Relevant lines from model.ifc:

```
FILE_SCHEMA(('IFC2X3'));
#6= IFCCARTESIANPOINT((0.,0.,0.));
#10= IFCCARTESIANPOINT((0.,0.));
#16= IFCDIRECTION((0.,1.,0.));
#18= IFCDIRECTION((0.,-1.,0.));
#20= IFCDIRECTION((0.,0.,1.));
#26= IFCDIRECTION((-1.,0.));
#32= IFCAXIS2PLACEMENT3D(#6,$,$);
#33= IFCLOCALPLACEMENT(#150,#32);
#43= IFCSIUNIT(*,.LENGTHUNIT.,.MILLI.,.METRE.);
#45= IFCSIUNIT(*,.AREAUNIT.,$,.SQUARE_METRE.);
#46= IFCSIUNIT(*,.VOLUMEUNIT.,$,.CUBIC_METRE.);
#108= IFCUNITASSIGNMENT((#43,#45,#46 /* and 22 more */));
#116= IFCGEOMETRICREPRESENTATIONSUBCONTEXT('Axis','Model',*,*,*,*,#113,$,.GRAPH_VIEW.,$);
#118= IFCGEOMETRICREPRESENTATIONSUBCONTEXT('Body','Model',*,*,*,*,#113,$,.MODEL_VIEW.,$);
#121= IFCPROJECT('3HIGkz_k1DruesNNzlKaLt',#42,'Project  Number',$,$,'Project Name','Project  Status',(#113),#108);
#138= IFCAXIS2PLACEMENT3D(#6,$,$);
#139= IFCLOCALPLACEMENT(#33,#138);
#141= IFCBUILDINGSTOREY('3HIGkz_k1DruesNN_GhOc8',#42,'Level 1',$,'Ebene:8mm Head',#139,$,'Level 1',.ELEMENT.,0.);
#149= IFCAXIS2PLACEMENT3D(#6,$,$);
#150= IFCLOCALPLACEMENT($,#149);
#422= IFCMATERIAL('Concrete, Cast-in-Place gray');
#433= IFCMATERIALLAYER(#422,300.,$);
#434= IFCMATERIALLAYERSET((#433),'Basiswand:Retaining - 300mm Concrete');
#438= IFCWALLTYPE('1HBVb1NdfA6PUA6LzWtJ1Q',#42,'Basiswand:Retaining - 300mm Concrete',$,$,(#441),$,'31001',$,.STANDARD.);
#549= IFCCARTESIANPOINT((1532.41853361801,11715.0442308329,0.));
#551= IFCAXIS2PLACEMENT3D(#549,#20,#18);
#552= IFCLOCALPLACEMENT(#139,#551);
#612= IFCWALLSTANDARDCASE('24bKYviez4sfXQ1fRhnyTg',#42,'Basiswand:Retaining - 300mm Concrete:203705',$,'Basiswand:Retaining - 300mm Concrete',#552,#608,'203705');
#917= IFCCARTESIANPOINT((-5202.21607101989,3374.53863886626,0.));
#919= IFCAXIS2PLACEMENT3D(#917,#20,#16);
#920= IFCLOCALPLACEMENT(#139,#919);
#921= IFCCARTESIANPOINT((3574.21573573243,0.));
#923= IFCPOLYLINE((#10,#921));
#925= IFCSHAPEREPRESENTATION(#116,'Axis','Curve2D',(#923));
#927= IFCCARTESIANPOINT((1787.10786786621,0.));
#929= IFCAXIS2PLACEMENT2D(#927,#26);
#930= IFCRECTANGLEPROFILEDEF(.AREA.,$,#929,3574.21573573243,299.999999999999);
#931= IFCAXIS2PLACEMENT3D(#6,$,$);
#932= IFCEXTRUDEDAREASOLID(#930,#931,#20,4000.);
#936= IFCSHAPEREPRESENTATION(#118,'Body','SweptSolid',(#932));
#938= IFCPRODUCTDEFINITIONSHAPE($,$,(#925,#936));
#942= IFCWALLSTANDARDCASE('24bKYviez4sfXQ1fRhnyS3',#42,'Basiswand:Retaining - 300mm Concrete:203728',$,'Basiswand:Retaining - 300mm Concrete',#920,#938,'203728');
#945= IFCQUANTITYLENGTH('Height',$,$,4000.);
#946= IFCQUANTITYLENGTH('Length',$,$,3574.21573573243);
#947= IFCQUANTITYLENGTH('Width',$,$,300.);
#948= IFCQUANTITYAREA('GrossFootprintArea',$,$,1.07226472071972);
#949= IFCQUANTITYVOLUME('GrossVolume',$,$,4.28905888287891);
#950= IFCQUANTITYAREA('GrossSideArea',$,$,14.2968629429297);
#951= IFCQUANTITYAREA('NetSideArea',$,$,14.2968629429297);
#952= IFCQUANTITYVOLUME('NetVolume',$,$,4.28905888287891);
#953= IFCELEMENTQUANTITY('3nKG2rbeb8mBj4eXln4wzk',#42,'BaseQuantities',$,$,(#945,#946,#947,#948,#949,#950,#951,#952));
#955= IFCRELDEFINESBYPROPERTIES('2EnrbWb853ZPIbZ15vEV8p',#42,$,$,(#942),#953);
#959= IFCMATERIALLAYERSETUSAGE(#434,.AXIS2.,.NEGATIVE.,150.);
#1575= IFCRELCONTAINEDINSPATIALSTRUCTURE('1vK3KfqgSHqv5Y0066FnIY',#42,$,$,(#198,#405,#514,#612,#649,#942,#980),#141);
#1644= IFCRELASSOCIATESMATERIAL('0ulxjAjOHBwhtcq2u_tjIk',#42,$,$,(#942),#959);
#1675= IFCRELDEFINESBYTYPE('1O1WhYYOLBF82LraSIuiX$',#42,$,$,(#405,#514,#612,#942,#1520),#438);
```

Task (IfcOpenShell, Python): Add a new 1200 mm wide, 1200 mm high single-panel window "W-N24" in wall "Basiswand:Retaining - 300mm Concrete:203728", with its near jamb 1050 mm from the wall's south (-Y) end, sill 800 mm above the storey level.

```python
import numpy as np
import ifcopenshell
import ifcopenshell.api.feature
import ifcopenshell.api.geometry
import ifcopenshell.api.pset
import ifcopenshell.api.root
import ifcopenshell.api.spatial
import ifcopenshell.api.type
import ifcopenshell.geom
import ifcopenshell.util.element
import ifcopenshell.util.placement
import ifcopenshell.util.representation
import ifcopenshell.util.shape
import ifcopenshell.util.unit

model = ifcopenshell.open("model.ifc")
unit_scale = ifcopenshell.util.unit.calculate_unit_scale(model)
area_scale = ifcopenshell.util.unit.calculate_unit_scale(model, "AREAUNIT")
volume_scale = ifcopenshell.util.unit.calculate_unit_scale(model, "VOLUMEUNIT")
settings = ifcopenshell.geom.settings()


def volume(element):
    """Net volume in cubic metres, openings subtracted."""
    shape = ifcopenshell.geom.create_shape(settings, element)
    return ifcopenshell.util.shape.get_volume(shape.geometry)


wall = model.by_id(942)
storey = ifcopenshell.util.element.get_container(wall, ifc_class="IfcBuildingStorey")
context = ifcopenshell.util.representation.get_context(model, "Model", "Body", "MODEL_VIEW")
before = volume(wall)

width, height, from_end, sill = 1.2, 1.2, 1.05, 0.8  # metres

# The wall runs along its own X axis, and the end named is its -X end.
wall_shape = ifcopenshell.geom.create_shape(settings, wall)
x, y, z = ifcopenshell.util.shape.get_vertices(wall_shape.geometry).T
start = x.min() + from_end
face, thickness = float(y.min()), float(y.max() - y.min())
wall_matrix = ifcopenshell.util.placement.get_local_placement(wall.ObjectPlacement)
level = ifcopenshell.util.placement.get_local_placement(storey.ObjectPlacement)[2, 3]


def in_wall(x, y):
    """Placement at x, y metres in the wall's axes, at sill height."""
    matrix = wall_matrix.copy()
    matrix[:, 3] = wall_matrix @ np.array([x / unit_scale, y / unit_scale, 0.0, 1.0])
    matrix[2, 3] = level + sill / unit_scale
    return matrix


# Opening: a box that overshoots both wall faces by 50 mm.
opening = ifcopenshell.api.root.create_entity(model, ifc_class="IfcOpeningElement")
box = ifcopenshell.api.geometry.add_wall_representation(
    model, context=context, length=width, height=height, thickness=thickness + 0.1
)
ifcopenshell.api.geometry.assign_representation(model, product=opening, representation=box)
ifcopenshell.api.geometry.edit_object_placement(model, product=opening, matrix=in_wall(start, face - 0.05), is_si=False)
ifcopenshell.api.feature.add_feature(model, feature=opening, element=wall)

window = ifcopenshell.api.root.create_entity(model, ifc_class="IfcWindow", name="W-N24")
window.OverallWidth, window.OverallHeight = width / unit_scale, height / unit_scale
body = ifcopenshell.api.geometry.add_window_representation(
    model,
    context=context,
    overall_width=window.OverallWidth,
    overall_height=window.OverallHeight,
    partition_type="SINGLE_PANEL",
)
ifcopenshell.api.geometry.assign_representation(model, product=window, representation=body)
ifcopenshell.api.spatial.assign_container(model, products=[window], relating_structure=storey)
fills = ifcopenshell.api.feature.add_filling(model, opening=opening, element=window)
fills.OwnerHistory = window.OwnerHistory  # required in IFC2X3

# IFC2X3 keeps the operation on the window style.
style = ifcopenshell.api.root.create_entity(model, ifc_class="IfcWindowStyle", name="W-N24")
style.OperationType, style.ConstructionType = "SINGLE_PANEL", "NOTDEFINED"
style.ParameterTakesPrecedence = style.Sizeable = False
ifcopenshell.api.type.assign_type(model, related_objects=[window], relating_type=style)

# Centre the window in the wall's thickness.
ifcopenshell.api.geometry.edit_object_placement(model, product=window, matrix=in_wall(start, face), is_si=False)
window_shape = ifcopenshell.geom.create_shape(settings, window)
depth = ifcopenshell.util.shape.get_vertices(window_shape.geometry)[:, 1]
offset = face + thickness / 2 - (depth.min() + depth.max()) / 2
ifcopenshell.api.geometry.edit_object_placement(model, product=window, matrix=in_wall(start, offset), is_si=False)

after = volume(wall)

# Update the wall's stored quantities.
qto = model.by_id(ifcopenshell.util.element.get_pset(wall, "BaseQuantities", should_inherit=False)["id"])
ifcopenshell.api.pset.edit_qto(model, qto=qto, properties={
    "NetSideArea": after / thickness / area_scale,
    "NetVolume": after / volume_scale,
})

print(f"wall volume {before:.3f} -> {after:.3f} m3")

model.write("model-out.ifc")
```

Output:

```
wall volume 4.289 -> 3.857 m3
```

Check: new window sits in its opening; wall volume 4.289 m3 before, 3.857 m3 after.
